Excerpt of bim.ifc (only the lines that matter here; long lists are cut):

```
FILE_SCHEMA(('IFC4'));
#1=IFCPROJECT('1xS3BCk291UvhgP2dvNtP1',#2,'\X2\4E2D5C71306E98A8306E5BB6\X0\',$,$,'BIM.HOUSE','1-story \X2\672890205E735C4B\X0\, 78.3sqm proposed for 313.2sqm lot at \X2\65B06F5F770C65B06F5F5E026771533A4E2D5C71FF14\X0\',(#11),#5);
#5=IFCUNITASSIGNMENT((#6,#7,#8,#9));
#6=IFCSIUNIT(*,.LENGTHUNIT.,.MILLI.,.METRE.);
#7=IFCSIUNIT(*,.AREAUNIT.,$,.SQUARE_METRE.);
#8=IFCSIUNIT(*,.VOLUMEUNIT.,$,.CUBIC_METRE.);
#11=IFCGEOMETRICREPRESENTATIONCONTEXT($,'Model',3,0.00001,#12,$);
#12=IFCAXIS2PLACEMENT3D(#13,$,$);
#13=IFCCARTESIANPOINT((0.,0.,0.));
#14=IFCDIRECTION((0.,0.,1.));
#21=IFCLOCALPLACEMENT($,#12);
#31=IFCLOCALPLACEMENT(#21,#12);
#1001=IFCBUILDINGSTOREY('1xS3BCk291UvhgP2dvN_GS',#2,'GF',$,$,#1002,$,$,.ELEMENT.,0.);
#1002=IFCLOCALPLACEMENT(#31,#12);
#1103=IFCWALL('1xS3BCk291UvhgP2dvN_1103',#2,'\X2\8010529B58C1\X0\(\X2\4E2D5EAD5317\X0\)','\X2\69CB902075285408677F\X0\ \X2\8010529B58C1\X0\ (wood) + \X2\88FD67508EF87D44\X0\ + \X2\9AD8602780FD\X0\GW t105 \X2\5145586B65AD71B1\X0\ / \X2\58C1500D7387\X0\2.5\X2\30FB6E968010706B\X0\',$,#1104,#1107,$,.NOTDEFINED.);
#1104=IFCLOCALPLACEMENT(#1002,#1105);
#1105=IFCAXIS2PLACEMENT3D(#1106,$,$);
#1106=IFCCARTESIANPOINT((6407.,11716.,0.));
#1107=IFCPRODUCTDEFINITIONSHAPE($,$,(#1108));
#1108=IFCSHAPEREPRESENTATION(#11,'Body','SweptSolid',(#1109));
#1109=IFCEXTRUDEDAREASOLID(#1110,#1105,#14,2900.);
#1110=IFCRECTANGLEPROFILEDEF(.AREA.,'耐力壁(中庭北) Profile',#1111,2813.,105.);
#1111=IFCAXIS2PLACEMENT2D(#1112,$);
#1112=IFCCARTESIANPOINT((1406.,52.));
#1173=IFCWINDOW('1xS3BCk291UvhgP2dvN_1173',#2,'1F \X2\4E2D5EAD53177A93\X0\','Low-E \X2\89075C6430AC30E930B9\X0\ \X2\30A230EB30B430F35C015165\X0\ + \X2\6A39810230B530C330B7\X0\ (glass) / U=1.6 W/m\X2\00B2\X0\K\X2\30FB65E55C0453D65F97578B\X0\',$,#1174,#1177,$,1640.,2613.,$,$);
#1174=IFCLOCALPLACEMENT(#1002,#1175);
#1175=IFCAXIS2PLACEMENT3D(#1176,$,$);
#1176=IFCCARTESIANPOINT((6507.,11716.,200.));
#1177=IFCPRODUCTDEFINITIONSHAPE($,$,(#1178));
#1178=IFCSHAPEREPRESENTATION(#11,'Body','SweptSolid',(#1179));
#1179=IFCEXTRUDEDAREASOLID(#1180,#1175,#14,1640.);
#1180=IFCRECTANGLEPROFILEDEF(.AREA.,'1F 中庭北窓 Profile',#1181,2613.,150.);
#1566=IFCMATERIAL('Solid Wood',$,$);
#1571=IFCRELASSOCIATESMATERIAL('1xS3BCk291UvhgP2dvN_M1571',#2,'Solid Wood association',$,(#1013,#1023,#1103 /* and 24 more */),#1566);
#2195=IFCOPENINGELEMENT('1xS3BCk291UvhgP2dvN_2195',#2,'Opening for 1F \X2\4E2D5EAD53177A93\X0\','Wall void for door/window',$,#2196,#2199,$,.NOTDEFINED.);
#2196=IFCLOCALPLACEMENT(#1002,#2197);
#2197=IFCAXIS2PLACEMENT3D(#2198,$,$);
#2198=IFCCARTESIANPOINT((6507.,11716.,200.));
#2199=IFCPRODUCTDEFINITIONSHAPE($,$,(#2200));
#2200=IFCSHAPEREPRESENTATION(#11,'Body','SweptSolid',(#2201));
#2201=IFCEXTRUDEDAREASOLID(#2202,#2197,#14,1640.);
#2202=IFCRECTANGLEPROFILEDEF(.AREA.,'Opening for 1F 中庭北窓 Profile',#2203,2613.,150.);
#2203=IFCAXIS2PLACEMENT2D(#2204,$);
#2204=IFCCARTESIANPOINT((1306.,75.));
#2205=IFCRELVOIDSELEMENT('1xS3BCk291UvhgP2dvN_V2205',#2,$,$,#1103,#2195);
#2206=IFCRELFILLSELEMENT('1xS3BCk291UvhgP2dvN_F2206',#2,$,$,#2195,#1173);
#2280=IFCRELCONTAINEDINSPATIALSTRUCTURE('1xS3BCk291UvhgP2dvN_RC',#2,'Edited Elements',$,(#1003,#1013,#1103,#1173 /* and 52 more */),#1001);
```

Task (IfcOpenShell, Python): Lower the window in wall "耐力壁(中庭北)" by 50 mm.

```python
import numpy as np
import ifcopenshell
import ifcopenshell.api.geometry
import ifcopenshell.util.placement
import ifcopenshell.util.unit

model = ifcopenshell.open("bim.ifc")
unit_scale = ifcopenshell.util.unit.calculate_unit_scale(model)

window = model.by_guid("1xS3BCk291UvhgP2dvN_1173")
opening = window.FillsVoids[0].RelatingOpeningElement
dz = -50.0

shift = np.array([0.0, 0.0, dz])
# The window is not placed relative to its opening, so move both.
for product in (opening, window):
    matrix = ifcopenshell.util.placement.get_local_placement(product.ObjectPlacement)
    matrix[:3, 3] += shift
    ifcopenshell.api.geometry.edit_object_placement(model, product=product, matrix=matrix, is_si=False)

print(f"moved by {dz * unit_scale:+.3f} m")

model.write("bim_v2.ifc")
```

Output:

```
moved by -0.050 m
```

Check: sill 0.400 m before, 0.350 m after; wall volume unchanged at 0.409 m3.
